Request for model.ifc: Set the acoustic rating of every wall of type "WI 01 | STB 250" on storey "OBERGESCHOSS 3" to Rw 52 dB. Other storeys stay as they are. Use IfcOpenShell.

First a look at what the model holds.

```python
import ifcopenshell
import ifcopenshell.util.element

model = ifcopenshell.open("model.ifc")
print(model.schema)
storey = next(s for s in model.by_type("IfcBuildingStorey") if s.Name == "OBERGESCHOSS 3")
walls = [e for e in ifcopenshell.util.element.get_decomposition(storey) if e.is_a("IfcWall")]
seen = {}
for e in walls:
    element_type = ifcopenshell.util.element.get_type(e)
    key = (element_type.Name if element_type != e and element_type else None, ifcopenshell.util.element.get_pset(e, "Pset_WallCommon", "AcousticRating"))
    seen[key] = seen.get(key, 0) + 1
for (name, value), count in sorted(seen.items(), key=str):
    print(count, "x", name, "|", value)
```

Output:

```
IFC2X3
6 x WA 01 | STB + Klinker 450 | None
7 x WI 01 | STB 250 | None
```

```python
import ifcopenshell
import ifcopenshell.api.pset
import ifcopenshell.util.element

model = ifcopenshell.open("model.ifc")

storey = next(s for s in model.by_type("IfcBuildingStorey") if s.Name == "OBERGESCHOSS 3")
walls = [e for e in ifcopenshell.util.element.get_decomposition(storey) if e.is_a("IfcWall")]

count = 0
for e in walls:
    element_type = ifcopenshell.util.element.get_type(e)
    if element_type in (None, e) or element_type.Name != 'WI\xa001 |\xa0STB 250':
        continue
    # add_pset returns the element's existing set when there is one.
    pset = ifcopenshell.api.pset.add_pset(model, product=e, name="Pset_WallCommon")
    ifcopenshell.api.pset.edit_pset(model, pset=pset, properties={"AcousticRating": "Rw 52 dB"})
    count += 1

print(count, "walls updated")

model.write("model_updated.ifc")
```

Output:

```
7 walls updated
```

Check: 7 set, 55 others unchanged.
